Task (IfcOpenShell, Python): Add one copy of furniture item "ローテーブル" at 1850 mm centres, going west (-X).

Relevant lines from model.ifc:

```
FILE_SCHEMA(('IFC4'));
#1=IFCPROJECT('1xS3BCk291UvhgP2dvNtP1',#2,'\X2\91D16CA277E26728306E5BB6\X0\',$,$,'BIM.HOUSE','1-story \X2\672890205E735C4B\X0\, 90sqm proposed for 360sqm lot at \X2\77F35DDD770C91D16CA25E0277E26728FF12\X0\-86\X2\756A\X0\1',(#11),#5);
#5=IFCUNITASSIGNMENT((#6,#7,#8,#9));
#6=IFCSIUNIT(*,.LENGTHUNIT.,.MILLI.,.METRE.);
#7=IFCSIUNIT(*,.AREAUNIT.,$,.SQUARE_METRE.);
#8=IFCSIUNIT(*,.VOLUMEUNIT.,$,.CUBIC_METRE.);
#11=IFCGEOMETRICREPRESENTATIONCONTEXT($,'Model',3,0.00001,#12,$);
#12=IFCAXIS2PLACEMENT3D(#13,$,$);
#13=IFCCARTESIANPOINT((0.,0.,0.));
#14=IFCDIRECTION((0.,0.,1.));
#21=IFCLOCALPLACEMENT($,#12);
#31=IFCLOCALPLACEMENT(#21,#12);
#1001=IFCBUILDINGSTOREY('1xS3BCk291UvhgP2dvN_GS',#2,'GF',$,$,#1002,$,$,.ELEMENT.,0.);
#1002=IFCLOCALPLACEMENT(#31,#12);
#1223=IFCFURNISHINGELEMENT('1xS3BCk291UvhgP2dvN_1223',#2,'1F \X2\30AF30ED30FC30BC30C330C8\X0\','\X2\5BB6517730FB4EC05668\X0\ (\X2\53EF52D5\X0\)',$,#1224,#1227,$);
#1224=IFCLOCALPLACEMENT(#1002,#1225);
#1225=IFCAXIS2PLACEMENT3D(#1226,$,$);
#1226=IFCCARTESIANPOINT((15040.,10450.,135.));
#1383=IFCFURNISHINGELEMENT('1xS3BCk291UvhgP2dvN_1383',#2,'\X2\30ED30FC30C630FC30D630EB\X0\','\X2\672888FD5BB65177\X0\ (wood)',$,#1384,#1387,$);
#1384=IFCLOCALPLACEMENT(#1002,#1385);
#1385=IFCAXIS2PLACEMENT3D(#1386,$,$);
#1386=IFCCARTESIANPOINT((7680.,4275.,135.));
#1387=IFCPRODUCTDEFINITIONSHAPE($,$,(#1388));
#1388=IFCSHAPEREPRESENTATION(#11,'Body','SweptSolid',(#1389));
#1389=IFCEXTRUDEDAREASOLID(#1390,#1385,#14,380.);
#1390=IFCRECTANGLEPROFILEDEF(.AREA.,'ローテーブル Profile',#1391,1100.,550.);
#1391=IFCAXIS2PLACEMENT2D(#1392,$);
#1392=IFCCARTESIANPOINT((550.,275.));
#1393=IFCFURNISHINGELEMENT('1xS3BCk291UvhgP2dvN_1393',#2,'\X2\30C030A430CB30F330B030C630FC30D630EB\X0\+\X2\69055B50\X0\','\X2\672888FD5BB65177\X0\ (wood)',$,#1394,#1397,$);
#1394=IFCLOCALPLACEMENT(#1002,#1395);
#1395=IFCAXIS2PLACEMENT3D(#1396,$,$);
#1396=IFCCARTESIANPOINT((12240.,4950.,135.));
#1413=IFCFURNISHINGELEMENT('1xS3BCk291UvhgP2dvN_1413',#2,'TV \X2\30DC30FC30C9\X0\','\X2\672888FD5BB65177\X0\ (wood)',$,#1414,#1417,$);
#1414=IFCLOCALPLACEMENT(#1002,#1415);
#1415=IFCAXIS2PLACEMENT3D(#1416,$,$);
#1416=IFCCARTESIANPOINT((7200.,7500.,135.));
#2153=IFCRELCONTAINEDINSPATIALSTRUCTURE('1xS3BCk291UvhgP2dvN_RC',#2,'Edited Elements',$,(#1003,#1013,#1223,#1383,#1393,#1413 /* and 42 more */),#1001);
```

```python
import numpy as np
import ifcopenshell
import ifcopenshell.api.geometry
import ifcopenshell.api.root
import ifcopenshell.util.element
import ifcopenshell.util.placement

model = ifcopenshell.open("model.ifc")


def reuse_history(source, copy):
    """copy_class also copies each property set's owner history, people and application; keep the originals."""
    for rel in copy.IsDefinedBy:
        if rel.is_a("IfcRelDefinesByProperties") and (history := rel.RelatingPropertyDefinition.OwnerHistory):
            rel.RelatingPropertyDefinition.OwnerHistory = source.OwnerHistory
            ifcopenshell.util.element.remove_deep2(model, history)


source = model.by_guid("1xS3BCk291UvhgP2dvN_1383")
base = ifcopenshell.util.placement.get_local_placement(source.ObjectPlacement)
step = np.array([-1.0, 0.0, 0.0]) * 1850.0

for i in range(1, 2):
    copy = ifcopenshell.api.root.copy_class(model, product=source)
    copy.Representation = ifcopenshell.util.element.copy_deep(
        model, source.Representation, exclude=["IfcGeometricRepresentationContext", "IfcRepresentationMap"]
    )
    reuse_history(source, copy)
    matrix = base.copy()
    matrix[:3, 3] += i * step
    print("added at", matrix[:3, 3].round(3) + 0.0)
    ifcopenshell.api.geometry.edit_object_placement(model, product=copy, matrix=matrix, is_si=False)

model.write("model_edited.ifc")
```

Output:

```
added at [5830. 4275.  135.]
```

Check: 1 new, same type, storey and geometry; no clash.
